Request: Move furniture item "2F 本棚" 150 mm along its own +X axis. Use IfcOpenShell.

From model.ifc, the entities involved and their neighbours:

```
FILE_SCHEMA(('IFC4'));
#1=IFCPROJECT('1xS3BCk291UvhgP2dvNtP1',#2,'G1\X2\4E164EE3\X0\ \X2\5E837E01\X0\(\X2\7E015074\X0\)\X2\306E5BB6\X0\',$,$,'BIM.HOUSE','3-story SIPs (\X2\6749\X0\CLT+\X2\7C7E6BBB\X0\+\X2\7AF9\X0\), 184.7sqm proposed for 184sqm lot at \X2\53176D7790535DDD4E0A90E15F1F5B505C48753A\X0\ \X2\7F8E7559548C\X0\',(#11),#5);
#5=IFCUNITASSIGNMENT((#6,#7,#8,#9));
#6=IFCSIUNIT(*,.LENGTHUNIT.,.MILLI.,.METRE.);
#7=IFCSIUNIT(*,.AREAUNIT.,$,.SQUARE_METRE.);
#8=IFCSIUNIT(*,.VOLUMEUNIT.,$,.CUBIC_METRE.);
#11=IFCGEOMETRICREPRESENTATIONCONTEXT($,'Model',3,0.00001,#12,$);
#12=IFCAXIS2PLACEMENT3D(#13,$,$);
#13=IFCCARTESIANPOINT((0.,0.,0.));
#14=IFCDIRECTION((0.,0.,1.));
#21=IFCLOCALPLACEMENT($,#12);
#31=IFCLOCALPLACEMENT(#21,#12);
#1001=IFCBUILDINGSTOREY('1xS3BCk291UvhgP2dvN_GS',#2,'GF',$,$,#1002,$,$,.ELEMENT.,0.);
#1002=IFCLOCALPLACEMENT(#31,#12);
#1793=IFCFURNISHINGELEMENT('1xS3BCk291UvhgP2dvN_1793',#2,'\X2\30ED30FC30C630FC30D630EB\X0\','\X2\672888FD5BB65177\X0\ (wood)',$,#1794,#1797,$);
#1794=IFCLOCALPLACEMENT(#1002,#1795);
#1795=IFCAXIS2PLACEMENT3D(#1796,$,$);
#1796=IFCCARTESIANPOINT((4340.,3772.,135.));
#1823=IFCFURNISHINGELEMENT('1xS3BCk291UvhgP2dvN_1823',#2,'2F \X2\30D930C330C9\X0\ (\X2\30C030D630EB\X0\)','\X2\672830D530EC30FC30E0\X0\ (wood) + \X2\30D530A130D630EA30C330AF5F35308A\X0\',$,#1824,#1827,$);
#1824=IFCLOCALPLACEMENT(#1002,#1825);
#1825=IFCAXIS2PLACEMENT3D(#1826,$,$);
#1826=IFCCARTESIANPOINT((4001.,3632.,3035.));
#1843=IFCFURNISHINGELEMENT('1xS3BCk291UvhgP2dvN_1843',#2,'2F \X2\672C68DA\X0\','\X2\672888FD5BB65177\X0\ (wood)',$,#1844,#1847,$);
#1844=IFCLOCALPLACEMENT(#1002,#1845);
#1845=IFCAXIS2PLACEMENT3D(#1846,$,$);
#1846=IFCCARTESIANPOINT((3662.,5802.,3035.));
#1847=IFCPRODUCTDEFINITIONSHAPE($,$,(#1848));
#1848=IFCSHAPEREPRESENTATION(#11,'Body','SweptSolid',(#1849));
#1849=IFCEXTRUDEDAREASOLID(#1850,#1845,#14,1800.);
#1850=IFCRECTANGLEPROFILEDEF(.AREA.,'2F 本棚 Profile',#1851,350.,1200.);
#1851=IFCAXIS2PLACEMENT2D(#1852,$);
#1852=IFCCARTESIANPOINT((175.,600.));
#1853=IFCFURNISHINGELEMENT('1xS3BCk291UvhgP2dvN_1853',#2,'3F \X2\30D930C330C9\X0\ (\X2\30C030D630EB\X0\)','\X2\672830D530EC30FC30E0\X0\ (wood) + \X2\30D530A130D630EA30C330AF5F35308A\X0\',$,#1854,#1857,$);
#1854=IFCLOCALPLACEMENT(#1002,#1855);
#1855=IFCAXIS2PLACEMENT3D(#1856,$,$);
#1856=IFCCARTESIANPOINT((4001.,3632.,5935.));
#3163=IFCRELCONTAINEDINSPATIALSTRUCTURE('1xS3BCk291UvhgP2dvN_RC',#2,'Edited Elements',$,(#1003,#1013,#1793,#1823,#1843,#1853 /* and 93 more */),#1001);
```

```python
import ifcopenshell
import ifcopenshell.api.geometry
import ifcopenshell.util.placement

model = ifcopenshell.open("model.ifc")

item = model.by_guid("1xS3BCk291UvhgP2dvN_1843")
matrix = ifcopenshell.util.placement.get_local_placement(item.ObjectPlacement)
matrix[:3, 3] += matrix[:3, 0] * 150.0
ifcopenshell.api.geometry.edit_object_placement(model, product=item, matrix=matrix, is_si=False)

print(ifcopenshell.util.placement.get_local_placement(item.ObjectPlacement).round(3) + 0.0)

model.write("model_rev.ifc")
```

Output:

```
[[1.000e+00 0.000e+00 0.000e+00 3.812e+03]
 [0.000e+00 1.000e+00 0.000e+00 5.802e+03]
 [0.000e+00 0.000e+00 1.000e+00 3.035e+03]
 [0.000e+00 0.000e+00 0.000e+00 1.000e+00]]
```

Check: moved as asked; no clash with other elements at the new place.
